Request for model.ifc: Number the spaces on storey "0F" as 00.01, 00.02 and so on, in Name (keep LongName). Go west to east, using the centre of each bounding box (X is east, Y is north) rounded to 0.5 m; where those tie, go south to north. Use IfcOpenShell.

First a look at what the model holds.

```python
import ifcopenshell
import ifcopenshell.util.element
import ifcopenshell.util.placement

model = ifcopenshell.open("model.ifc")
print(model.schema)
storey = next(s for s in model.by_type("IfcBuildingStorey") if s.Name == "0F")
spaces = [e for e in ifcopenshell.util.element.get_decomposition(storey) if e.is_a("IfcSpace")]
for e in sorted(spaces, key=lambda e: e.id()):
    origin = ifcopenshell.util.placement.get_local_placement(e.ObjectPlacement)[:3, 3]
    print(e.id(), e.Name, e.LongName, origin.round(2) + 0.0, sep=" | ")
```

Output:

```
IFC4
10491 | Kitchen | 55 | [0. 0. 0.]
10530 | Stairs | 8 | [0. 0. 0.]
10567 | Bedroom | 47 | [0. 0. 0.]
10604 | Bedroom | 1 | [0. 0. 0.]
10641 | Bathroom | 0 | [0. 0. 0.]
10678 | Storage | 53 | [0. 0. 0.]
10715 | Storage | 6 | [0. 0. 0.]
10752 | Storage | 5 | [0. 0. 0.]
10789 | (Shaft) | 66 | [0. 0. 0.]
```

```python
import ifcopenshell
import ifcopenshell.geom
import ifcopenshell.util.element
import ifcopenshell.util.shape

model = ifcopenshell.open("model.ifc")
settings = ifcopenshell.geom.settings()
settings.set("use-world-coords", True)


def centre(element):
    shape = ifcopenshell.geom.create_shape(settings, element)
    return ifcopenshell.util.shape.get_bbox_centroid(shape.geometry)


storey = next(s for s in model.by_type("IfcBuildingStorey") if s.Name == "0F")
spaces = [e for e in ifcopenshell.util.element.get_decomposition(storey) if e.is_a("IfcSpace")]

# Insertion points can sit at a corner or the storey origin, so sort by the geometry (in metres).
centres = {e: centre(e) for e in spaces}
spaces.sort(key=lambda e: (round(centres[e][0] / 0.5), centres[e][1]))

for i, e in enumerate(spaces, start=1):
    number = f"00.{i:02d}"
    e.Name = number
    print(e.id(), number)

model.write("model-out.ifc")
```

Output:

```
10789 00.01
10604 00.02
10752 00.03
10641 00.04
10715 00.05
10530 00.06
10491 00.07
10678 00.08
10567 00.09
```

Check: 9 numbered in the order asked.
